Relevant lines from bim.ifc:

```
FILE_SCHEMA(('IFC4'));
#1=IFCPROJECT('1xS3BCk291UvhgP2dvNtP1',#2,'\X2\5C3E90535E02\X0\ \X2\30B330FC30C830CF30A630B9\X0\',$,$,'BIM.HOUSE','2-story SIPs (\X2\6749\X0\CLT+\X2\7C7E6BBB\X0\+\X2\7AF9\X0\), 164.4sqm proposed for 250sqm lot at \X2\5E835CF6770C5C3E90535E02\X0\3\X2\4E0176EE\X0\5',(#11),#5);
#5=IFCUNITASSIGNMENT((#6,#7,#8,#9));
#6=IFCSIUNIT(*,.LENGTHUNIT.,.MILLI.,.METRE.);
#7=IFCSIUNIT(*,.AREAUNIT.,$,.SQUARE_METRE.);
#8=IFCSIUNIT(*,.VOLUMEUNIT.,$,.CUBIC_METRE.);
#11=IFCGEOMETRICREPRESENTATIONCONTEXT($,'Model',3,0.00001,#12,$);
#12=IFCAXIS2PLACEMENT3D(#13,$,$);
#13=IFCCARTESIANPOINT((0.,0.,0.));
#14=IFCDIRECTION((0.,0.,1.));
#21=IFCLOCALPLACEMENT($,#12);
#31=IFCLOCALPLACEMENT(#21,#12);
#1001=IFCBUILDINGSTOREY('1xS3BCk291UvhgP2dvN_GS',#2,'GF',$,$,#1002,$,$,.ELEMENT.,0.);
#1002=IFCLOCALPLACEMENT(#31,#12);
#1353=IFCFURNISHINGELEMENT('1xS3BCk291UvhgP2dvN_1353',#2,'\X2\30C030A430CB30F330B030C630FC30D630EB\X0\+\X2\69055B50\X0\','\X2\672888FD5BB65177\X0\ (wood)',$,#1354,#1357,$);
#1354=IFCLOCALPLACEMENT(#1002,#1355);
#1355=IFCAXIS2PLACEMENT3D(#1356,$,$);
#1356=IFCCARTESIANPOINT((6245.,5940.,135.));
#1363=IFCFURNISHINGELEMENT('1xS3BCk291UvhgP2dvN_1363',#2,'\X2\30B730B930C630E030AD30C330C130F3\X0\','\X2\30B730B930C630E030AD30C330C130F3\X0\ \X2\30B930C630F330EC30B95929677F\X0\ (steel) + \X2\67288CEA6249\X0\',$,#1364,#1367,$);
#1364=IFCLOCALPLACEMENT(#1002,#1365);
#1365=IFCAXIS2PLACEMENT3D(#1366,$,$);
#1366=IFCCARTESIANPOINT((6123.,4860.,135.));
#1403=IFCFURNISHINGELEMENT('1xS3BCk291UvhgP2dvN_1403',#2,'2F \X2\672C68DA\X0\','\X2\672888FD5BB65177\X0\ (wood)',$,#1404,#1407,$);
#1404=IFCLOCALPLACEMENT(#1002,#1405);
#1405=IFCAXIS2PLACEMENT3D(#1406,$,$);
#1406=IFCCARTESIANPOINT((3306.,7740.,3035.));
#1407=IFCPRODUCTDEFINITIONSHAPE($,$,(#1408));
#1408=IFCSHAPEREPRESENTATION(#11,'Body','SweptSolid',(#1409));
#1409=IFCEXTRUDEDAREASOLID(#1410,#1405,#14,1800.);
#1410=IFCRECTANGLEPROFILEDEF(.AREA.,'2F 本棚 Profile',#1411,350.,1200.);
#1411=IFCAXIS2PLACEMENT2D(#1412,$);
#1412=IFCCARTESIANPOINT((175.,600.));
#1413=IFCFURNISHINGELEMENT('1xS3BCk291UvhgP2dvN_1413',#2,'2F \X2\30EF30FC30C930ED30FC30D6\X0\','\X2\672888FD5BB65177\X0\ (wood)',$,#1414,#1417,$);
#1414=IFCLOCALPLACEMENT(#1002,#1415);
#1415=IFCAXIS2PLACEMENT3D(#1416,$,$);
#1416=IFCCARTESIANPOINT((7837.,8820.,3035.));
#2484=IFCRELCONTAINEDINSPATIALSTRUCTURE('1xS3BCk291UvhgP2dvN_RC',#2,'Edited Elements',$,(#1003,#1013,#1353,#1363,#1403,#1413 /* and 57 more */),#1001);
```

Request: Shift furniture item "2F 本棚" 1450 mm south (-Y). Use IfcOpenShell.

```python
import ifcopenshell
import ifcopenshell.api.geometry
import ifcopenshell.util.placement
import ifcopenshell.util.unit

model = ifcopenshell.open("bim.ifc")
unit_scale = ifcopenshell.util.unit.calculate_unit_scale(model)

item = model.by_guid("1xS3BCk291UvhgP2dvN_1403")
matrix = ifcopenshell.util.placement.get_local_placement(item.ObjectPlacement)
matrix[1, 3] -= 1.45 / unit_scale
ifcopenshell.api.geometry.edit_object_placement(model, product=item, matrix=matrix, is_si=False)

print(ifcopenshell.util.placement.get_local_placement(item.ObjectPlacement).round(3) + 0.0)

model.write("bim_rev.ifc")
```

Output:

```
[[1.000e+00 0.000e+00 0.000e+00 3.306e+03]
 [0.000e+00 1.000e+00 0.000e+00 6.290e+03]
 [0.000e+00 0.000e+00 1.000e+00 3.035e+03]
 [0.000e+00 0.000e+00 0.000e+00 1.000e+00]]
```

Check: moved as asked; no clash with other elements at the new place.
